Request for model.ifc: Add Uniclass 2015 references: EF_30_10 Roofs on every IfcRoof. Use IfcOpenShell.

First a look at what the model holds.

```python
import ifcopenshell

model = ifcopenshell.open("model.ifc")
print(model.schema)
print("classifications:", [c.Name for c in model.by_type("IfcClassification")])
for ifc_class in ("IfcDoor", "IfcRoof", "IfcStair", "IfcWall", "IfcWindow"):
    print(ifc_class, len(model.by_type(ifc_class)))
```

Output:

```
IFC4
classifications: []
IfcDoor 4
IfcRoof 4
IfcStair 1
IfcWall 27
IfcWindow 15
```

```python
import ifcopenshell
import ifcopenshell.api.classification

model = ifcopenshell.open("model.ifc")

system = ifcopenshell.api.classification.add_classification(model, classification="Uniclass 2015")

codes = {
    "IfcRoof": ("EF_30_10", "Roofs"),
}
for ifc_class, (code, name) in codes.items():
    products = model.by_type(ifc_class)
    ifcopenshell.api.classification.add_reference(
        model, products=products, classification=system, identification=code, name=name
    )
    print(code, len(products))

model.write("model_updated.ifc")
```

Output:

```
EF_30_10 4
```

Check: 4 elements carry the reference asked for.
